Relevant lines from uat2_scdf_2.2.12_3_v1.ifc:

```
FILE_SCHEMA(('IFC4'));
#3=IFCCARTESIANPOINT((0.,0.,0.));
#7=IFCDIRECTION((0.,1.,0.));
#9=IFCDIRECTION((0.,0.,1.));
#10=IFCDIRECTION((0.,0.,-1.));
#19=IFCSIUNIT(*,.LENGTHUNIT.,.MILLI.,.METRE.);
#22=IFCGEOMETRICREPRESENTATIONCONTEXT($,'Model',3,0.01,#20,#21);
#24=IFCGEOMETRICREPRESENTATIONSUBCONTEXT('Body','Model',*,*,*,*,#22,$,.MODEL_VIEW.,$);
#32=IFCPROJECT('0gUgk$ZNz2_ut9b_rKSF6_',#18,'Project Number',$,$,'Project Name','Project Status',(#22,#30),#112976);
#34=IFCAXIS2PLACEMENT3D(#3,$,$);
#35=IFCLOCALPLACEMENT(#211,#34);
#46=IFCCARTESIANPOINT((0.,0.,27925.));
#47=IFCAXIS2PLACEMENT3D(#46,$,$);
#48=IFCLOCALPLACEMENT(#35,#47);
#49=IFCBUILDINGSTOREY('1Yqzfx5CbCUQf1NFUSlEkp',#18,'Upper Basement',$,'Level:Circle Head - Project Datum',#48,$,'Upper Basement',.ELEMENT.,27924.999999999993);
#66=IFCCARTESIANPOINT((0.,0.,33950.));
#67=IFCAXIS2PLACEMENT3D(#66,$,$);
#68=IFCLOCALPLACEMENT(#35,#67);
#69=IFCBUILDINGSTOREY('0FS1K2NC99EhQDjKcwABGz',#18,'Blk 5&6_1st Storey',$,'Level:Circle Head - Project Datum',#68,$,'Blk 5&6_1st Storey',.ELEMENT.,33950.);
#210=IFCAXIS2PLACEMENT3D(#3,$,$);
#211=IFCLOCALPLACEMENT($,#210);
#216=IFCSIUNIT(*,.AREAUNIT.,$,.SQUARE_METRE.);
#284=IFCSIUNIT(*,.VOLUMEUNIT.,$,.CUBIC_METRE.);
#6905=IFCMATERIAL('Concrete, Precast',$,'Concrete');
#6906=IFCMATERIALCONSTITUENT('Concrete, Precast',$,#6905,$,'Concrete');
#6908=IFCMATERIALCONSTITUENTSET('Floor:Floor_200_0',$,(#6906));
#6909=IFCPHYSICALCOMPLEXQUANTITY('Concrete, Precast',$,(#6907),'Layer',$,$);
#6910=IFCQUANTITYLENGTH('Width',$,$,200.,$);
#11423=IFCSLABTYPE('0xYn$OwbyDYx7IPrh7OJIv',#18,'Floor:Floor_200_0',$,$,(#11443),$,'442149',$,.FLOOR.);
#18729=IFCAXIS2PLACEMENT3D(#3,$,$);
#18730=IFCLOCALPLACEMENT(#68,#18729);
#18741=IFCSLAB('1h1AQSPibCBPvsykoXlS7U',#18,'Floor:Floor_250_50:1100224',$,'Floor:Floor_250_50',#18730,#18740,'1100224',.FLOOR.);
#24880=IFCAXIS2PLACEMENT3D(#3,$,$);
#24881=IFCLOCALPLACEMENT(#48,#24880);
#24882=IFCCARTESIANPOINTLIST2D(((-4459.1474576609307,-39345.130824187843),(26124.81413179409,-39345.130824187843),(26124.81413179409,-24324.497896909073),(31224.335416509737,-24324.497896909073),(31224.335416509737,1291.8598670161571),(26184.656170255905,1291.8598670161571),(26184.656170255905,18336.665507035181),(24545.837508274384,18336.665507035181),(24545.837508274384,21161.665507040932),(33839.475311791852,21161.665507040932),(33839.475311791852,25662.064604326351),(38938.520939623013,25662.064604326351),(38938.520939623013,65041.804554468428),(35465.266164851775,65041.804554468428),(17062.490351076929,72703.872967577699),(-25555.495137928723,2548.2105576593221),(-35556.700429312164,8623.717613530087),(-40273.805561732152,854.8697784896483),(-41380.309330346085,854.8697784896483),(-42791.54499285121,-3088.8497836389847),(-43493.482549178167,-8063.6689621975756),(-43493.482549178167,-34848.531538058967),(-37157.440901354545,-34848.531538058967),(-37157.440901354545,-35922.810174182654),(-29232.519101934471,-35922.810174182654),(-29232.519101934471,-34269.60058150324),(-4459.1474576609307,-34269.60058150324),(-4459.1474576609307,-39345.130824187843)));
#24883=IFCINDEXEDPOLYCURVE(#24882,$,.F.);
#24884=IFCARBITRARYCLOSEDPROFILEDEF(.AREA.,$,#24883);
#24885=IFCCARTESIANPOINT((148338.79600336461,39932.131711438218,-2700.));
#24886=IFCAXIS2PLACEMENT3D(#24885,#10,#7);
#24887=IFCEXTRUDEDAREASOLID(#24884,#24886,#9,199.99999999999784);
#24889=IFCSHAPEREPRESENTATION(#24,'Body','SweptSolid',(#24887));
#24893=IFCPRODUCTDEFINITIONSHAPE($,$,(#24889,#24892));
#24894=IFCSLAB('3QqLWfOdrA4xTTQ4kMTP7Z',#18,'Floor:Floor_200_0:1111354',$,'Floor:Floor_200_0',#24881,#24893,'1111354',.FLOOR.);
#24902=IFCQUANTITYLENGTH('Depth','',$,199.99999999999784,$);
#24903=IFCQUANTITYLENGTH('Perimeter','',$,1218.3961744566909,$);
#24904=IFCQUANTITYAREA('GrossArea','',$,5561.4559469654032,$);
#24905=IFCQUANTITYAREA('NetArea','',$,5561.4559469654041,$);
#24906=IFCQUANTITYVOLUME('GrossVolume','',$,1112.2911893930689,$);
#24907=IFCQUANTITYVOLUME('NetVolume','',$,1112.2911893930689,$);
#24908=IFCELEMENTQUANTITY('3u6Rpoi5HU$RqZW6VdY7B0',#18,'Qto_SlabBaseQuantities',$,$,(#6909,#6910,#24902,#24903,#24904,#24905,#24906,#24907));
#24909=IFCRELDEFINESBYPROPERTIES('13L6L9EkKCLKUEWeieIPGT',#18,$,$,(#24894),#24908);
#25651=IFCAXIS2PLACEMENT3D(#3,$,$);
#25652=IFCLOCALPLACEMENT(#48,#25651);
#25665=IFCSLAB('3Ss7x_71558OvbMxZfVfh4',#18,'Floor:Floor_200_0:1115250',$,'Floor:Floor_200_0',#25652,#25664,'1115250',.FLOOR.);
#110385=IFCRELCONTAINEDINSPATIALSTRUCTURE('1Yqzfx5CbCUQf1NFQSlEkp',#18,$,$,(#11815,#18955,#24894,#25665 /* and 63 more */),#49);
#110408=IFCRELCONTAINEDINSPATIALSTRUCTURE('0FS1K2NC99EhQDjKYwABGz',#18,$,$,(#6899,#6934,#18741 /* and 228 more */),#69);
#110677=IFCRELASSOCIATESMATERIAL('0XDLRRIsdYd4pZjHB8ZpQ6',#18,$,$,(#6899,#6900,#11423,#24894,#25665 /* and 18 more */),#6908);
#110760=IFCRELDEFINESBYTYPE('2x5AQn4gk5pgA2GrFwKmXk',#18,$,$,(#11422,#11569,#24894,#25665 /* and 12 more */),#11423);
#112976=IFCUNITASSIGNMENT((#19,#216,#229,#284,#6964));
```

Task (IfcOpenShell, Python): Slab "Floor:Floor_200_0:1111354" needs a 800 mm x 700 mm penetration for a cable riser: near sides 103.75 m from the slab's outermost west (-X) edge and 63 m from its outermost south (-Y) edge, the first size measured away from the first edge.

```python
import numpy as np
import ifcopenshell
import ifcopenshell.api.feature
import ifcopenshell.api.geometry
import ifcopenshell.api.pset
import ifcopenshell.api.root
import ifcopenshell.geom
import ifcopenshell.util.element
import ifcopenshell.util.placement
import ifcopenshell.util.representation
import ifcopenshell.util.shape
import ifcopenshell.util.unit

model = ifcopenshell.open("uat2_scdf_2.2.12_3_v1.ifc")
unit_scale = ifcopenshell.util.unit.calculate_unit_scale(model)
area_scale = ifcopenshell.util.unit.calculate_unit_scale(model, "AREAUNIT")
volume_scale = ifcopenshell.util.unit.calculate_unit_scale(model, "VOLUMEUNIT")
settings = ifcopenshell.geom.settings()


def volume(element):
    """Net volume in cubic metres, openings subtracted."""
    shape = ifcopenshell.geom.create_shape(settings, element)
    return ifcopenshell.util.shape.get_volume(shape.geometry)


slab = model.by_guid("3QqLWfOdrA4xTTQ4kMTP7Z")
before = volume(slab)

# Extent in the slab's own axes, in metres. The edges named are its -X and -Y sides.
slab_shape = ifcopenshell.geom.create_shape(settings, slab)
vertices = ifcopenshell.util.shape.get_vertices(slab_shape.geometry)
x_min, y_min, bottom = vertices.min(axis=0)
top = vertices[:, 2].max()

opening = ifcopenshell.api.root.create_entity(model, ifc_class="IfcOpeningElement", name="Cable riser opening", predefined_type="OPENING")
context = ifcopenshell.util.representation.get_context(model, "Model", "Body", "MODEL_VIEW")
width, depth = 0.8, 0.7
outline = [(0.0, 0.0), (width, 0.0), (width, depth), (0.0, depth), (0.0, 0.0)]
# Overshoot both faces by 50 mm so the cut is clean.
shape = ifcopenshell.api.geometry.add_slab_representation(
    model, context=context, depth=top - bottom + 0.1, polyline=outline
)
ifcopenshell.api.geometry.assign_representation(model, product=opening, representation=shape)

matrix = ifcopenshell.util.placement.get_local_placement(slab.ObjectPlacement)
matrix[:, 3] = matrix @ np.append(np.array([x_min + 103.75, y_min + 63, bottom - 0.05]) / unit_scale, 1.0)
ifcopenshell.api.geometry.edit_object_placement(model, product=opening, matrix=matrix, is_si=False)
ifcopenshell.api.feature.add_feature(model, feature=opening, element=slab)

after = volume(slab)

# Update the slab's stored quantities.
qto = model.by_id(ifcopenshell.util.element.get_pset(slab, "Qto_SlabBaseQuantities", should_inherit=False)["id"])
ifcopenshell.api.pset.edit_qto(model, qto=qto, properties={
    "NetArea": after / (top - bottom) / area_scale,
    "NetVolume": after / volume_scale,
})

print(f"slab volume {before:.3f} -> {after:.3f} m3")

model.write("uat2_scdf_2.2.12_3_v1_rev.ifc")
```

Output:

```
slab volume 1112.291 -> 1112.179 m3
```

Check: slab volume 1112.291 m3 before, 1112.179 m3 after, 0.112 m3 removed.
